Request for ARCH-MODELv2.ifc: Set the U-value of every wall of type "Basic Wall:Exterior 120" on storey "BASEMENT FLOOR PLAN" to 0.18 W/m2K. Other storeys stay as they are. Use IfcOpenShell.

First a look at what the model holds.

```python
import ifcopenshell
import ifcopenshell.util.element

model = ifcopenshell.open("ARCH-MODELv2.ifc")
print(model.schema)
storey = next(s for s in model.by_type("IfcBuildingStorey") if s.Name == "BASEMENT FLOOR PLAN")
walls = [e for e in ifcopenshell.util.element.get_decomposition(storey) if e.is_a("IfcWall")]
seen = {}
for e in walls:
    element_type = ifcopenshell.util.element.get_type(e)
    key = (element_type.Name if element_type != e and element_type else None, ifcopenshell.util.element.get_pset(e, "Pset_WallCommon", "ThermalTransmittance"))
    seen[key] = seen.get(key, 0) + 1
for (name, value), count in sorted(seen.items(), key=str):
    print(count, "x", name, "|", value)
```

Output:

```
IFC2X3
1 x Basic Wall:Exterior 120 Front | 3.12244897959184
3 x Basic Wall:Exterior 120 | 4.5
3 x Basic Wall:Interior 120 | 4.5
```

```python
import ifcopenshell
import ifcopenshell.api.pset
import ifcopenshell.util.element

model = ifcopenshell.open("ARCH-MODELv2.ifc")

storey = next(s for s in model.by_type("IfcBuildingStorey") if s.Name == "BASEMENT FLOOR PLAN")
walls = [e for e in ifcopenshell.util.element.get_decomposition(storey) if e.is_a("IfcWall")]

count = 0
for e in walls:
    element_type = ifcopenshell.util.element.get_type(e)
    if element_type in (None, e) or element_type.Name != "Basic Wall:Exterior 120":
        continue
    # add_pset returns the element's existing set when there is one.
    pset = ifcopenshell.api.pset.add_pset(model, product=e, name="Pset_WallCommon")
    ifcopenshell.api.pset.edit_pset(model, pset=pset, properties={"ThermalTransmittance": 0.18})
    count += 1

print(count, "walls updated")

model.write("ARCH-MODELv2-out.ifc")
```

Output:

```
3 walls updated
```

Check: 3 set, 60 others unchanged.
